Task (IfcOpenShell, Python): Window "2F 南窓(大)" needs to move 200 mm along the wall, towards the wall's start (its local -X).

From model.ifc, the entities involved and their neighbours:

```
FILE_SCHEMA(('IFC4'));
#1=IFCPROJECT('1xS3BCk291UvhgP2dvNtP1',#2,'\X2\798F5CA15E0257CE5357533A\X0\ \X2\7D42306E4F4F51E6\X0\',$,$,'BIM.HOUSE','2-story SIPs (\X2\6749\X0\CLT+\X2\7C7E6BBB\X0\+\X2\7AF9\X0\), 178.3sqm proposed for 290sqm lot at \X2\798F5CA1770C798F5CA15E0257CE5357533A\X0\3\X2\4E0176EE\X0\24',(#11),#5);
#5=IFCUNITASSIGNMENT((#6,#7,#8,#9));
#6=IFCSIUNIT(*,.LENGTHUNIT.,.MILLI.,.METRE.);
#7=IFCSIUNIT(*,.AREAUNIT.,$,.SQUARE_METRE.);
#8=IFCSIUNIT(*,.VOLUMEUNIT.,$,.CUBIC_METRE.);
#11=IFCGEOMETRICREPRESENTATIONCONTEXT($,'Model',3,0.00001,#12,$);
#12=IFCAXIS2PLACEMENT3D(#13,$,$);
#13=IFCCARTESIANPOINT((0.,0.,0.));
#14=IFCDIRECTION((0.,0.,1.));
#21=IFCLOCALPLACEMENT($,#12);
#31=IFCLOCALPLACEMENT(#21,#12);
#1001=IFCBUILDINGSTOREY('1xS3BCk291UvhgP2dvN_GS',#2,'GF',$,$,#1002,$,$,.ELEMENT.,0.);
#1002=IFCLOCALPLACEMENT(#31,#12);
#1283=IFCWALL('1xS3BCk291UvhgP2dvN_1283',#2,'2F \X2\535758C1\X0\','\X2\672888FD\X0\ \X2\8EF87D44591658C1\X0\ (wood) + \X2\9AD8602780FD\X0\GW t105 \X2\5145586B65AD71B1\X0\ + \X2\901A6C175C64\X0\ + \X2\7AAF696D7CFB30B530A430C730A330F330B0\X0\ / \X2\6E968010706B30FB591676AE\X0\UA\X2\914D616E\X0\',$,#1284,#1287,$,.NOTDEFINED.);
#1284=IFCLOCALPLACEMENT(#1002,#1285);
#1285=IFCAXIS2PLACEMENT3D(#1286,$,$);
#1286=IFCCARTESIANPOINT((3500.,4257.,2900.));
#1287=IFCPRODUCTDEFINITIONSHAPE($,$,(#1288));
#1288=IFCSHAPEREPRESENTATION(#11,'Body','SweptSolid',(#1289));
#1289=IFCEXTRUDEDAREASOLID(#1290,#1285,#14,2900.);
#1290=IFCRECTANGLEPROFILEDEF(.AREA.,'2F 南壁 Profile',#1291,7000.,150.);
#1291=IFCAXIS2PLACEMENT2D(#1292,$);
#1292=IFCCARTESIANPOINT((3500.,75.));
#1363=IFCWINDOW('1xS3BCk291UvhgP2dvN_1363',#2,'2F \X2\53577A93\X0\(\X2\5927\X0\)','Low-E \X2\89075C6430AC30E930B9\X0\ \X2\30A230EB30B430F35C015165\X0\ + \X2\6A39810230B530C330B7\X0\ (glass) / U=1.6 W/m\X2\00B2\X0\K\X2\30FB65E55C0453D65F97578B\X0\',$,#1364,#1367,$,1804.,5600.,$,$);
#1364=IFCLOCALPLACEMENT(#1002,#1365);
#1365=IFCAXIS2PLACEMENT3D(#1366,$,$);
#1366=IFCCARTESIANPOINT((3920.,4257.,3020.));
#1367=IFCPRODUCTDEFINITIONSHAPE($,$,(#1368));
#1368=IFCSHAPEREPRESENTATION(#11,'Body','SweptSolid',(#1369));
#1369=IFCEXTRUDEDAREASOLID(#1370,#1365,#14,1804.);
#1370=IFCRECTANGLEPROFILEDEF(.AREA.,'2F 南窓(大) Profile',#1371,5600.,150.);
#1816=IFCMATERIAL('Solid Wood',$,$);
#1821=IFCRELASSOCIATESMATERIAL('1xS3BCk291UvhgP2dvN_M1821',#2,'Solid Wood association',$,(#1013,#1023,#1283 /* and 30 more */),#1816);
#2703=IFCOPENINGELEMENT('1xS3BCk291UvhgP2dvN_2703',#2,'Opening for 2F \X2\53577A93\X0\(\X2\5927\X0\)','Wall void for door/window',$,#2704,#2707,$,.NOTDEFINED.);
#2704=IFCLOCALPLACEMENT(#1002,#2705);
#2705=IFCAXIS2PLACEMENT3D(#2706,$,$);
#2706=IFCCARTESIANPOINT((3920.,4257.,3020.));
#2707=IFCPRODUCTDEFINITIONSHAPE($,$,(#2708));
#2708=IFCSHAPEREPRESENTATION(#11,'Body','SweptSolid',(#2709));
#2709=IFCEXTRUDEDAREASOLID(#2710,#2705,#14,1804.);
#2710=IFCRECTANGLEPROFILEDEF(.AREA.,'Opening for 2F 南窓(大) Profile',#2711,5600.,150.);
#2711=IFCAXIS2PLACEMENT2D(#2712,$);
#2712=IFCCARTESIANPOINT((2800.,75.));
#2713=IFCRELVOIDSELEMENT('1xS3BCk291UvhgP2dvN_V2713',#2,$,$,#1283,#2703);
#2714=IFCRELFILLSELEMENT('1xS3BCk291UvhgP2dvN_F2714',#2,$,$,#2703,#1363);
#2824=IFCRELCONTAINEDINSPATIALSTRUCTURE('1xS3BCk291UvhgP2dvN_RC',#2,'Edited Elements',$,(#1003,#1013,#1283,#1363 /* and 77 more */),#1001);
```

```python
import ifcopenshell
import ifcopenshell.api.geometry
import ifcopenshell.util.placement
import ifcopenshell.util.unit

model = ifcopenshell.open("model.ifc")
unit_scale = ifcopenshell.util.unit.calculate_unit_scale(model)

window = model.by_guid("1xS3BCk291UvhgP2dvN_1363")
opening = window.FillsVoids[0].RelatingOpeningElement
wall = opening.VoidsElements[0].RelatingBuildingElement

wall_matrix = ifcopenshell.util.placement.get_local_placement(wall.ObjectPlacement)
shift = wall_matrix[:3, 0] * -0.2 / unit_scale
before = ifcopenshell.util.placement.get_local_placement(window.ObjectPlacement)[:3, 3].copy()

# The window is not placed relative to its opening, so move both.
for product in (opening, window):
    matrix = ifcopenshell.util.placement.get_local_placement(product.ObjectPlacement)
    matrix[:3, 3] += shift
    ifcopenshell.api.geometry.edit_object_placement(model, product=product, matrix=matrix, is_si=False)

after = ifcopenshell.util.placement.get_local_placement(window.ObjectPlacement)[:3, 3]
print("window moved by", (after - before).round(3) + 0.0)

model.write("model-out.ifc")
```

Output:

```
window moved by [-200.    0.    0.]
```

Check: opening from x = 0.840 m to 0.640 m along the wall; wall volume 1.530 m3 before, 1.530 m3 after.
